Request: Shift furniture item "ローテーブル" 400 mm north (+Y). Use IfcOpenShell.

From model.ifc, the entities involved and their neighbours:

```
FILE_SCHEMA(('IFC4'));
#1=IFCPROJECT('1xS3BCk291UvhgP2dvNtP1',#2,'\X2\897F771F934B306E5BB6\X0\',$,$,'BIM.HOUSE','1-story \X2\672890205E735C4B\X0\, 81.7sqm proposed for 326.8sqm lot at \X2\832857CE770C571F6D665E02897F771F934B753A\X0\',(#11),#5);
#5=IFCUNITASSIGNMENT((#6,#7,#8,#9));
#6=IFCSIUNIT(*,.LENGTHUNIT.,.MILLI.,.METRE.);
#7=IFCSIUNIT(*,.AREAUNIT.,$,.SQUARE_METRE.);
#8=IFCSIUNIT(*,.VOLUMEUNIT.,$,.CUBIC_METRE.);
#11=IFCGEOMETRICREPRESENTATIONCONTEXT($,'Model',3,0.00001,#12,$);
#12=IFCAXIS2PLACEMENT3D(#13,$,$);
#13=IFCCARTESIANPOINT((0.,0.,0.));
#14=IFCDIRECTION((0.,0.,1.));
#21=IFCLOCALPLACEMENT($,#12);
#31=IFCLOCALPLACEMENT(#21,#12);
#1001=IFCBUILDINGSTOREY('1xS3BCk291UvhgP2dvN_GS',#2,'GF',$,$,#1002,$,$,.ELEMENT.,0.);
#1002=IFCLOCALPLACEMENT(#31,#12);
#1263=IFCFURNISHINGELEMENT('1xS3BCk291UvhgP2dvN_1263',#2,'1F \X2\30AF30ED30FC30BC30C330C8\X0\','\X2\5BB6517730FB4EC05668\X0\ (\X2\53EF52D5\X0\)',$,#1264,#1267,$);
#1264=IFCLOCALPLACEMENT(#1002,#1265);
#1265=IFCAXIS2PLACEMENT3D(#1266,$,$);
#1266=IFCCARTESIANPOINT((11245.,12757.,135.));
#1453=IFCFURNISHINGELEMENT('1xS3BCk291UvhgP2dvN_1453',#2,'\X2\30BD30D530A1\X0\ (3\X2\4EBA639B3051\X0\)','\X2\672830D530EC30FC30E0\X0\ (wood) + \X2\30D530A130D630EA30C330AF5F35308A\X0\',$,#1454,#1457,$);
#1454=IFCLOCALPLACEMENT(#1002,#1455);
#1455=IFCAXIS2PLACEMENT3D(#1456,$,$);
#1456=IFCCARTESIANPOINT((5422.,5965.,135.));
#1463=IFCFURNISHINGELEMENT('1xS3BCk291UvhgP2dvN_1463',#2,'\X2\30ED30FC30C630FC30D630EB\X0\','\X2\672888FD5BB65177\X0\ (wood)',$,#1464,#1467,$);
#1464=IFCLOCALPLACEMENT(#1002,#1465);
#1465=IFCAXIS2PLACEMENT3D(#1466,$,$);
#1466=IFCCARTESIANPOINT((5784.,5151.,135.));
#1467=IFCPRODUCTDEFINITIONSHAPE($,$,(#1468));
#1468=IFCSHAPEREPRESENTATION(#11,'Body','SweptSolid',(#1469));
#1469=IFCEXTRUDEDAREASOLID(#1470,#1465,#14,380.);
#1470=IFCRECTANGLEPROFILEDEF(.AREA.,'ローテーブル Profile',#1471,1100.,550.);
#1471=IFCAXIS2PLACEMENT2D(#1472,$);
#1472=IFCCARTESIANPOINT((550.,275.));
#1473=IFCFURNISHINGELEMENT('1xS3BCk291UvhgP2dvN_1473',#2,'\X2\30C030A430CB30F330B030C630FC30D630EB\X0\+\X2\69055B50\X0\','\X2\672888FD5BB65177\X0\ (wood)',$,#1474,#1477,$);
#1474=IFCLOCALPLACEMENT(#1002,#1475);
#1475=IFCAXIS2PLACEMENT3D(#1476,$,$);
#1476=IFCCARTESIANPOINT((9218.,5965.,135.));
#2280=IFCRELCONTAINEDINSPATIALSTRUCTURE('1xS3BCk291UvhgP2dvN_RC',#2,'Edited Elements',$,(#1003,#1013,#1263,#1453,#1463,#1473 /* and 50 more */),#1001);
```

```python
import ifcopenshell
import ifcopenshell.api.geometry
import ifcopenshell.util.placement

model = ifcopenshell.open("model.ifc")

item = model.by_guid("1xS3BCk291UvhgP2dvN_1463")
matrix = ifcopenshell.util.placement.get_local_placement(item.ObjectPlacement)
matrix[1, 3] += 400.0
ifcopenshell.api.geometry.edit_object_placement(model, product=item, matrix=matrix, is_si=False)

print(ifcopenshell.util.placement.get_local_placement(item.ObjectPlacement).round(3) + 0.0)

model.write("model_v2.ifc")
```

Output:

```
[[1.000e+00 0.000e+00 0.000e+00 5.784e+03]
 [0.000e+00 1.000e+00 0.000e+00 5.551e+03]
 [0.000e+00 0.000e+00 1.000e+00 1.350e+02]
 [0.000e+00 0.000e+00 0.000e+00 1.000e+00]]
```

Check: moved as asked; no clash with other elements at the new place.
